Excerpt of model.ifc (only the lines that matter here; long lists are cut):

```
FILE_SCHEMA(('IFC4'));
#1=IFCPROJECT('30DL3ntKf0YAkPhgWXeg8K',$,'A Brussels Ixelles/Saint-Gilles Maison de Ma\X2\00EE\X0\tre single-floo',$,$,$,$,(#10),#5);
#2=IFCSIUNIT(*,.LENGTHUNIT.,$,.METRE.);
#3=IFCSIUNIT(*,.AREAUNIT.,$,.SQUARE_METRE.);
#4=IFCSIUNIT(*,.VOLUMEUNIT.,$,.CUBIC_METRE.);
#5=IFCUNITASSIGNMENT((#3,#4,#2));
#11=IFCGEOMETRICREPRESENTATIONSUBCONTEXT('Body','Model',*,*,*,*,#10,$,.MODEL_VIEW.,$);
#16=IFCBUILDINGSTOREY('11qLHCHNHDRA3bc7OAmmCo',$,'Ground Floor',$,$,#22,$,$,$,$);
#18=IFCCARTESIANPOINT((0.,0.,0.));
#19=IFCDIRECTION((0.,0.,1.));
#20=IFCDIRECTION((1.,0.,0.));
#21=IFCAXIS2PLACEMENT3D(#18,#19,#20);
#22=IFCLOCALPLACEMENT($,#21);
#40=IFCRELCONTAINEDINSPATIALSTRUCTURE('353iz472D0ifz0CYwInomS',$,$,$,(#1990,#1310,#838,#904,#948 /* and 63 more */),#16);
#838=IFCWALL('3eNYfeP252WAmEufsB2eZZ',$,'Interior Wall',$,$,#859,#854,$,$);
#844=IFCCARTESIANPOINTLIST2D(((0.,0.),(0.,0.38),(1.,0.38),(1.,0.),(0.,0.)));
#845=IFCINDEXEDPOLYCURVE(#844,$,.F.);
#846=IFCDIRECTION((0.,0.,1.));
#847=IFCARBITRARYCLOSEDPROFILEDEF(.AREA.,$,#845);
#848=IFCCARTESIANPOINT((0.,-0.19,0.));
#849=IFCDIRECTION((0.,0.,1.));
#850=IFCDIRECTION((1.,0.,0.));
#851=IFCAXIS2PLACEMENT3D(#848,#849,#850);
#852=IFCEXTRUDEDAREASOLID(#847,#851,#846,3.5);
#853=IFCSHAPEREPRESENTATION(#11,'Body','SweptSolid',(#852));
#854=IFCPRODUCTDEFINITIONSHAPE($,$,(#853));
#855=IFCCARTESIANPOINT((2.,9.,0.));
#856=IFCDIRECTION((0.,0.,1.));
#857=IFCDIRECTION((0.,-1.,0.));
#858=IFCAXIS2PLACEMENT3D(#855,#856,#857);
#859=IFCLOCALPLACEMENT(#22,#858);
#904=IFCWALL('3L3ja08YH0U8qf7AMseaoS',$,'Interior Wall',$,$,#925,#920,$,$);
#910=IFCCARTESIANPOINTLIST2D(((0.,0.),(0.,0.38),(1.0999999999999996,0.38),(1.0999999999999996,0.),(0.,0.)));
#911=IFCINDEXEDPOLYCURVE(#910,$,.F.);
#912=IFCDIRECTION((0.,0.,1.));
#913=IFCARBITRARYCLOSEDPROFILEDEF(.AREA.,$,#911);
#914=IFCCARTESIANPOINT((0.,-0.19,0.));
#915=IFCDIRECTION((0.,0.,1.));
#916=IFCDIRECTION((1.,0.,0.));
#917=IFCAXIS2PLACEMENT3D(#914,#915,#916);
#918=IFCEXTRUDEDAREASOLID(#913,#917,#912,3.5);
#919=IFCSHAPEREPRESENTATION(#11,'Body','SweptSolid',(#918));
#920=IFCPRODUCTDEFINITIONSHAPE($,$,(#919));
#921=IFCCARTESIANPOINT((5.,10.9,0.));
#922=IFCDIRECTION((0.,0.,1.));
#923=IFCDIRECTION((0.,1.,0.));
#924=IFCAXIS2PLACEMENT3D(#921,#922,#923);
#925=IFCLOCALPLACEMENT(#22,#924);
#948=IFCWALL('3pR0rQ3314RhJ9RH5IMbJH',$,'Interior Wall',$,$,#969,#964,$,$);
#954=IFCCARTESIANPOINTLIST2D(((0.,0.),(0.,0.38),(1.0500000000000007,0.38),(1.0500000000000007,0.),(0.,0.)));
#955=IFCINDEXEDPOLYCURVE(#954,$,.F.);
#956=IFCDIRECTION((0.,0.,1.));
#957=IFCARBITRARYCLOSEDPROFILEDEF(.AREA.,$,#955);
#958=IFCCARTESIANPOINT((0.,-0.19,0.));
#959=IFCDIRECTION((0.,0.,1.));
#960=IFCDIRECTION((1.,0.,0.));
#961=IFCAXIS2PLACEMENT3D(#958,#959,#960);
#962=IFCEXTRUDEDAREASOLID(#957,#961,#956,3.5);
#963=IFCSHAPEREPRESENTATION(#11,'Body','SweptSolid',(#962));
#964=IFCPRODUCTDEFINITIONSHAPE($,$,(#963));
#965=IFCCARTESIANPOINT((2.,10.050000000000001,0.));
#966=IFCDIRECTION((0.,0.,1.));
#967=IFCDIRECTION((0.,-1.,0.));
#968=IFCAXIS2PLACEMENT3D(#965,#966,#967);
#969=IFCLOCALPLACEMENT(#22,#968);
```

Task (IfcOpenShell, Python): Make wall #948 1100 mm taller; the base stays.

```python
import ifcopenshell
import ifcopenshell.geom
import ifcopenshell.util.representation
import ifcopenshell.util.shape
import ifcopenshell.util.unit

model = ifcopenshell.open("model.ifc")
unit_scale = ifcopenshell.util.unit.calculate_unit_scale(model)
settings = ifcopenshell.geom.settings()


def volume(element):
    """Net volume in cubic metres, openings subtracted."""
    shape = ifcopenshell.geom.create_shape(settings, element)
    return ifcopenshell.util.shape.get_volume(shape.geometry)


wall = model.by_guid("3pR0rQ3314RhJ9RH5IMbJH")
before = volume(wall)

body = ifcopenshell.util.representation.get_representation(wall, "Model", "Body")
solid = body.Items[0]
old_height = solid.Depth
solid.Depth += 1.1 / unit_scale
after = volume(wall)

print(f"height {old_height:g} -> {solid.Depth:g}, volume {before:.3f} -> {after:.3f} m3")

model.write("model_rev.ifc")
```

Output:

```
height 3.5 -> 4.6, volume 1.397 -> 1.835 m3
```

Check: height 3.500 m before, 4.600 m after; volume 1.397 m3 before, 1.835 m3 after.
